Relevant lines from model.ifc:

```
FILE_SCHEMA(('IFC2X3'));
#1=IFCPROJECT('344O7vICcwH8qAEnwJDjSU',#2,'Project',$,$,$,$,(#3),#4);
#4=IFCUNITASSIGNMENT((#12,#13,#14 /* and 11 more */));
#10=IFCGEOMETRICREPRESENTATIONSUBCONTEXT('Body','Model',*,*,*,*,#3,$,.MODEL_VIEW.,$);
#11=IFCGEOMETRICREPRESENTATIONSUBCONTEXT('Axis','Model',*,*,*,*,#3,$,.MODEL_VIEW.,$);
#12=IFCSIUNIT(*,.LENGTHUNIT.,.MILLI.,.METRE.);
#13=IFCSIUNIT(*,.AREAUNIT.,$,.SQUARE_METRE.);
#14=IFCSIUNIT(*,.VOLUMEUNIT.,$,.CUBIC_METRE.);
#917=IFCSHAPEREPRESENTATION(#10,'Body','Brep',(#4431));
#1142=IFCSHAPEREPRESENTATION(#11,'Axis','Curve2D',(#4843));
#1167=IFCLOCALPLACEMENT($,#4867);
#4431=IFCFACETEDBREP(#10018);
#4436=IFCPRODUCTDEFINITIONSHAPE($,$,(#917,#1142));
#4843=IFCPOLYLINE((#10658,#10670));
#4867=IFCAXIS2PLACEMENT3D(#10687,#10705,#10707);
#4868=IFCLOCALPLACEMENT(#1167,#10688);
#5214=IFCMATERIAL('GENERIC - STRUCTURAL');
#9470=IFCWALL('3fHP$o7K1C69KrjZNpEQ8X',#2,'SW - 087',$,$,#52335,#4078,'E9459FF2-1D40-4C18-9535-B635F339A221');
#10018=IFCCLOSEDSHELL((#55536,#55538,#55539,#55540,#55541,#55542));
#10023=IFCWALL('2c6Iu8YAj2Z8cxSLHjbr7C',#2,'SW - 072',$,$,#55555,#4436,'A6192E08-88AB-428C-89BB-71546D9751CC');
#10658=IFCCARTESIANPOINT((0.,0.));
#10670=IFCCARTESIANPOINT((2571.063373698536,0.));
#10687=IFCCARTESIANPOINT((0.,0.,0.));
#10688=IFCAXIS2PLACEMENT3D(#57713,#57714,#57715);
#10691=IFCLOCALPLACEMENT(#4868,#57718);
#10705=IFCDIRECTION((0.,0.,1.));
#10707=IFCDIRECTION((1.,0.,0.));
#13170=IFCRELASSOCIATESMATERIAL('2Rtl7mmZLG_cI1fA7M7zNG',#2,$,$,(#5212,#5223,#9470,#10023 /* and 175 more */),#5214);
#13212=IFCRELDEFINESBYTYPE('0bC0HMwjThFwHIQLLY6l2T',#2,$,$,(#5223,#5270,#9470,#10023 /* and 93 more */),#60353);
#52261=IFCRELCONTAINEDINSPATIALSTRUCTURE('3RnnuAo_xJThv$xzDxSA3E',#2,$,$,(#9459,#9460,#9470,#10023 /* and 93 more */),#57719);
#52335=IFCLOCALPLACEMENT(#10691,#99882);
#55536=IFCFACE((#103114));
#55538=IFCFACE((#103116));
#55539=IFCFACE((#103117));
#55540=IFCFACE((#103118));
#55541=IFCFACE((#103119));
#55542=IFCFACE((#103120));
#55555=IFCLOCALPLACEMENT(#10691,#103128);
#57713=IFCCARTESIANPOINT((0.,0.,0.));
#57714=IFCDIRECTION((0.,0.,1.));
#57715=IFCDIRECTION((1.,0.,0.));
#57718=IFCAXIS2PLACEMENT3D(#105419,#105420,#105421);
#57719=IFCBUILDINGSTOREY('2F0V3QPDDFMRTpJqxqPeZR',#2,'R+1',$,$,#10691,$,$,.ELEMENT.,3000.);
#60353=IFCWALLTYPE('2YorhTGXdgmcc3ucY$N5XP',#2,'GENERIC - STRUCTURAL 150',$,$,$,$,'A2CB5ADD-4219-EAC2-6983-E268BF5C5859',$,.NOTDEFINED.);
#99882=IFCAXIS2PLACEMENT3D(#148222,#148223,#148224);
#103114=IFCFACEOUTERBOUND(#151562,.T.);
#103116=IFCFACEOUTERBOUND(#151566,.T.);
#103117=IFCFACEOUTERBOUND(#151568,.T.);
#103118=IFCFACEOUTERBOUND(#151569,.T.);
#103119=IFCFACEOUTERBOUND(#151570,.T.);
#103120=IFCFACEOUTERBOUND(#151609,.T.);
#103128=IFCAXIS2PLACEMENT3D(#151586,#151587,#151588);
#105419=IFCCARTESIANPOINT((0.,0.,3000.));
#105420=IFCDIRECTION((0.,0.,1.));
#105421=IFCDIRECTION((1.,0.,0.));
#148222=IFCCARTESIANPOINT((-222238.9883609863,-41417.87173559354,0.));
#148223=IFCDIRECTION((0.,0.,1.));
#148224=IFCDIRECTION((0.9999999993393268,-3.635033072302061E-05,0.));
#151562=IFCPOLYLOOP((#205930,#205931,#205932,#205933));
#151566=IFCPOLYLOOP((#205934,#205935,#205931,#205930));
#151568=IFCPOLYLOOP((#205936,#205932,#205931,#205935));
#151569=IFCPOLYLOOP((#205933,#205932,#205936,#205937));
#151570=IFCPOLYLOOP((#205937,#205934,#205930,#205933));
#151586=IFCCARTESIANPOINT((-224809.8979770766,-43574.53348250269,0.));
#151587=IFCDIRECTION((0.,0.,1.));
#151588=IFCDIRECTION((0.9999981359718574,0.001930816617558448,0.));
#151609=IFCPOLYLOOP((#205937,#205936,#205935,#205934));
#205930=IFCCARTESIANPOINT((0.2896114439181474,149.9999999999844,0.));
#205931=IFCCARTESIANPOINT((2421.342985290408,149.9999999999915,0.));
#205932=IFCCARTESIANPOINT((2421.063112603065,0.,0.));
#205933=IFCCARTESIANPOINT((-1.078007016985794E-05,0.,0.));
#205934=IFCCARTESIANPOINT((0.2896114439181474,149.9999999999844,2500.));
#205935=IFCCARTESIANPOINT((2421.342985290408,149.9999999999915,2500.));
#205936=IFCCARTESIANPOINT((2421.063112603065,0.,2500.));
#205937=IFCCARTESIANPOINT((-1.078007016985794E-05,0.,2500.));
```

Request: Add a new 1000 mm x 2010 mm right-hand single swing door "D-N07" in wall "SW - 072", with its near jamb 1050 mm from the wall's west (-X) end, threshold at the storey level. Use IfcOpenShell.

```python
import numpy as np
import ifcopenshell
import ifcopenshell.api.feature
import ifcopenshell.api.geometry
import ifcopenshell.api.root
import ifcopenshell.api.spatial
import ifcopenshell.api.type
import ifcopenshell.geom
import ifcopenshell.util.element
import ifcopenshell.util.placement
import ifcopenshell.util.representation
import ifcopenshell.util.shape
import ifcopenshell.util.unit

model = ifcopenshell.open("model.ifc")
unit_scale = ifcopenshell.util.unit.calculate_unit_scale(model)
settings = ifcopenshell.geom.settings()


def volume(element):
    """Net volume in cubic metres, openings subtracted."""
    shape = ifcopenshell.geom.create_shape(settings, element)
    return ifcopenshell.util.shape.get_volume(shape.geometry)


wall = model.by_guid("2c6Iu8YAj2Z8cxSLHjbr7C")
storey = ifcopenshell.util.element.get_container(wall, ifc_class="IfcBuildingStorey")
context = ifcopenshell.util.representation.get_context(model, "Model", "Body", "MODEL_VIEW")
before = volume(wall)

width, height, from_end, sill = 1, 2.01, 1.05, 0.0  # metres

# The wall runs along its own X axis, and the end named is its -X end.
wall_shape = ifcopenshell.geom.create_shape(settings, wall)
x, y, z = ifcopenshell.util.shape.get_vertices(wall_shape.geometry).T
start = x.min() + from_end
face, thickness = float(y.min()), float(y.max() - y.min())
wall_matrix = ifcopenshell.util.placement.get_local_placement(wall.ObjectPlacement)
level = ifcopenshell.util.placement.get_local_placement(storey.ObjectPlacement)[2, 3]


def in_wall(x, y):
    """Placement at x, y metres in the wall's axes, at sill height."""
    matrix = wall_matrix.copy()
    matrix[:, 3] = wall_matrix @ np.array([x / unit_scale, y / unit_scale, 0.0, 1.0])
    matrix[2, 3] = level + sill / unit_scale
    return matrix


# Opening: a box that overshoots both wall faces by 50 mm.
opening = ifcopenshell.api.root.create_entity(model, ifc_class="IfcOpeningElement")
box = ifcopenshell.api.geometry.add_wall_representation(
    model, context=context, length=width, height=height, thickness=thickness + 0.1
)
ifcopenshell.api.geometry.assign_representation(model, product=opening, representation=box)
ifcopenshell.api.geometry.edit_object_placement(model, product=opening, matrix=in_wall(start, face - 0.05), is_si=False)
ifcopenshell.api.feature.add_feature(model, feature=opening, element=wall)

door = ifcopenshell.api.root.create_entity(model, ifc_class="IfcDoor", name="D-N07")
door.OverallWidth, door.OverallHeight = width / unit_scale, height / unit_scale
body = ifcopenshell.api.geometry.add_door_representation(
    model,
    context=context,
    overall_width=door.OverallWidth,
    overall_height=door.OverallHeight,
    operation_type="SINGLE_SWING_RIGHT",
    lining_properties={"LiningDepth": thickness / unit_scale, "ThresholdDepth": thickness / unit_scale},
)
ifcopenshell.api.geometry.assign_representation(model, product=door, representation=body)
ifcopenshell.api.spatial.assign_container(model, products=[door], relating_structure=storey)
fills = ifcopenshell.api.feature.add_filling(model, opening=opening, element=door)
fills.OwnerHistory = door.OwnerHistory  # required in IFC2X3

# IFC2X3 keeps the operation on the door style.
style = ifcopenshell.api.root.create_entity(model, ifc_class="IfcDoorStyle", name="D-N07")
style.OperationType, style.ConstructionType = "SINGLE_SWING_RIGHT", "NOTDEFINED"
style.ParameterTakesPrecedence = style.Sizeable = False
ifcopenshell.api.type.assign_type(model, related_objects=[door], relating_type=style)

# The lining spans the wall, so the door starts at the wall face.
ifcopenshell.api.geometry.edit_object_placement(model, product=door, matrix=in_wall(start, face), is_si=False)

after = volume(wall)

print(f"wall volume {before:.3f} -> {after:.3f} m3")

model.write("model_v2.ifc")
```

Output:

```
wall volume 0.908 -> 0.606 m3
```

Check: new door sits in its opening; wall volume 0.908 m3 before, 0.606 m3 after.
